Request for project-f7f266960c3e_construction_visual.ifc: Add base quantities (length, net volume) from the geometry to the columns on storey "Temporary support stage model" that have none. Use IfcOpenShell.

First a look at what the model holds.

```python
import ifcopenshell
import ifcopenshell.util.element
import ifcopenshell.util.unit

model = ifcopenshell.open("project-f7f266960c3e_construction_visual.ifc")
print(model.schema)
for unit_type in ("LENGTHUNIT", "AREAUNIT", "VOLUMEUNIT"):
    print(unit_type, ifcopenshell.util.unit.calculate_unit_scale(model, unit_type))
storey = next(s for s in model.by_type("IfcBuildingStorey") if s.Name == "Temporary support stage model")
columns = [e for e in ifcopenshell.util.element.get_decomposition(storey) if e.is_a("IfcColumn")]
for e in sorted(columns, key=lambda e: e.id()):
    print(e.id(), e.is_a(), e.Name, list(ifcopenshell.util.element.get_psets(e, qtos_only=True)), sep=" | ")
```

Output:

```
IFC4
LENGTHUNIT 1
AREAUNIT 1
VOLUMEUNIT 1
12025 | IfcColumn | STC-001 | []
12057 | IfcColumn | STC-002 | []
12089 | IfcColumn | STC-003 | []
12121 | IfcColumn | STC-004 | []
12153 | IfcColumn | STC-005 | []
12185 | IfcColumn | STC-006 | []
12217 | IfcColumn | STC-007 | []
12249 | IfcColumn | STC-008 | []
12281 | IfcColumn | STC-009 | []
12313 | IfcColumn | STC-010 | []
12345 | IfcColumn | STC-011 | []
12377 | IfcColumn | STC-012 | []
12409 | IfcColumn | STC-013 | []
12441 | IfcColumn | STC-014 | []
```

```python
import ifcopenshell
import ifcopenshell.api.pset
import ifcopenshell.geom
import ifcopenshell.util.element
import ifcopenshell.util.shape
import ifcopenshell.util.unit

model = ifcopenshell.open("project-f7f266960c3e_construction_visual.ifc")
unit_scale = ifcopenshell.util.unit.calculate_unit_scale(model)
volume_scale = ifcopenshell.util.unit.calculate_unit_scale(model, "VOLUMEUNIT")
settings = ifcopenshell.geom.settings()

storey = next(s for s in model.by_type("IfcBuildingStorey") if s.Name == "Temporary support stage model")
columns = [e for e in ifcopenshell.util.element.get_decomposition(storey) if e.is_a("IfcColumn")]

for e in sorted(columns, key=lambda e: e.id()):
    if ifcopenshell.util.element.get_psets(e, qtos_only=True, should_inherit=False):
        continue
    # Geometry comes back in metres, in the element's own axes.
    shape = ifcopenshell.geom.create_shape(settings, e)
    values = {
        "Length": ifcopenshell.util.shape.get_z(shape.geometry) / unit_scale,
        "NetVolume": ifcopenshell.util.shape.get_volume(shape.geometry) / volume_scale,
    }
    qto = ifcopenshell.api.pset.add_qto(model, product=e, name="Qto_ColumnBaseQuantities")
    ifcopenshell.api.pset.edit_qto(model, qto=qto, properties=values)
    print(e.id(), {k: round(v, 3) for k, v in values.items()})

model.write("project-f7f266960c3e_construction_visual_edited.ifc")
```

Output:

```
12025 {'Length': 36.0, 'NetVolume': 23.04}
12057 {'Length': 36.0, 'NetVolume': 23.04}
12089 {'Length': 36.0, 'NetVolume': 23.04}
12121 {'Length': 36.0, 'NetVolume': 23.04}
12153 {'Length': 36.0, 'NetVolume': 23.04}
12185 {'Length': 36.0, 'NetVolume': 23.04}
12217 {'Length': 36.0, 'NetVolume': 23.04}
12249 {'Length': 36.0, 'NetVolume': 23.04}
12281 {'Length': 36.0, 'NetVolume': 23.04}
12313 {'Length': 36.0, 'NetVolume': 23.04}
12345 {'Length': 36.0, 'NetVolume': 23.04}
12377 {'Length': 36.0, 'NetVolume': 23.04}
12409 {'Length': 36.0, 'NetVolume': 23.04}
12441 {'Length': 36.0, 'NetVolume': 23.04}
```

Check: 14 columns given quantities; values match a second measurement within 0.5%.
